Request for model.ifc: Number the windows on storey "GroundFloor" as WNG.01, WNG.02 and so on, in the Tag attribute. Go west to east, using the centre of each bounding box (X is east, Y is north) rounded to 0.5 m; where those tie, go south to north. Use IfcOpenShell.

First a look at what the model holds.

```python
import ifcopenshell
import ifcopenshell.util.element
import ifcopenshell.util.placement

model = ifcopenshell.open("model.ifc")
print(model.schema)
storey = next(s for s in model.by_type("IfcBuildingStorey") if s.Name == "GroundFloor")
windows = [e for e in ifcopenshell.util.element.get_decomposition(storey) if e.is_a("IfcWindow")]
for e in sorted(windows, key=lambda e: e.id()):
    origin = ifcopenshell.util.placement.get_local_placement(e.ObjectPlacement)[:3, 3]
    print(e.id(), e.Tag, e.Name, origin.round(2) + 0.0, sep=" | ")
```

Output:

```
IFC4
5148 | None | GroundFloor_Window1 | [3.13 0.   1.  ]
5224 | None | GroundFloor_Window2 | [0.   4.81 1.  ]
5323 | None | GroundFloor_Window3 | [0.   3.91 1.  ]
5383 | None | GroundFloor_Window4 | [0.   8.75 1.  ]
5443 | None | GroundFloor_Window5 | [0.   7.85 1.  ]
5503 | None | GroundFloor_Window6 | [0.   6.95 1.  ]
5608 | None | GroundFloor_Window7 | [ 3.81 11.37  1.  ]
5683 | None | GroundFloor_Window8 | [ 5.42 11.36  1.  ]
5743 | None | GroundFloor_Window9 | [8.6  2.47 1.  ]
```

```python
import ifcopenshell
import ifcopenshell.geom
import ifcopenshell.util.element
import ifcopenshell.util.shape

model = ifcopenshell.open("model.ifc")
settings = ifcopenshell.geom.settings()
settings.set("use-world-coords", True)


def centre(element):
    shape = ifcopenshell.geom.create_shape(settings, element)
    return ifcopenshell.util.shape.get_bbox_centroid(shape.geometry)


storey = next(s for s in model.by_type("IfcBuildingStorey") if s.Name == "GroundFloor")
windows = [e for e in ifcopenshell.util.element.get_decomposition(storey) if e.is_a("IfcWindow")]

# Insertion points can sit at a corner or the storey origin, so sort by the geometry (in metres).
centres = {e: centre(e) for e in windows}
windows.sort(key=lambda e: (round(centres[e][0] / 0.5), centres[e][1]))

for i, e in enumerate(windows, start=1):
    number = f"WNG.{i:02d}"
    e.Tag = number
    print(e.id(), number)

model.write("model-out.ifc")
```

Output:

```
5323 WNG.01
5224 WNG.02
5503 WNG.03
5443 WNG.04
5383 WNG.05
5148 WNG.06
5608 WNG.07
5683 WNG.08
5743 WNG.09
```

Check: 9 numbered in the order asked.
